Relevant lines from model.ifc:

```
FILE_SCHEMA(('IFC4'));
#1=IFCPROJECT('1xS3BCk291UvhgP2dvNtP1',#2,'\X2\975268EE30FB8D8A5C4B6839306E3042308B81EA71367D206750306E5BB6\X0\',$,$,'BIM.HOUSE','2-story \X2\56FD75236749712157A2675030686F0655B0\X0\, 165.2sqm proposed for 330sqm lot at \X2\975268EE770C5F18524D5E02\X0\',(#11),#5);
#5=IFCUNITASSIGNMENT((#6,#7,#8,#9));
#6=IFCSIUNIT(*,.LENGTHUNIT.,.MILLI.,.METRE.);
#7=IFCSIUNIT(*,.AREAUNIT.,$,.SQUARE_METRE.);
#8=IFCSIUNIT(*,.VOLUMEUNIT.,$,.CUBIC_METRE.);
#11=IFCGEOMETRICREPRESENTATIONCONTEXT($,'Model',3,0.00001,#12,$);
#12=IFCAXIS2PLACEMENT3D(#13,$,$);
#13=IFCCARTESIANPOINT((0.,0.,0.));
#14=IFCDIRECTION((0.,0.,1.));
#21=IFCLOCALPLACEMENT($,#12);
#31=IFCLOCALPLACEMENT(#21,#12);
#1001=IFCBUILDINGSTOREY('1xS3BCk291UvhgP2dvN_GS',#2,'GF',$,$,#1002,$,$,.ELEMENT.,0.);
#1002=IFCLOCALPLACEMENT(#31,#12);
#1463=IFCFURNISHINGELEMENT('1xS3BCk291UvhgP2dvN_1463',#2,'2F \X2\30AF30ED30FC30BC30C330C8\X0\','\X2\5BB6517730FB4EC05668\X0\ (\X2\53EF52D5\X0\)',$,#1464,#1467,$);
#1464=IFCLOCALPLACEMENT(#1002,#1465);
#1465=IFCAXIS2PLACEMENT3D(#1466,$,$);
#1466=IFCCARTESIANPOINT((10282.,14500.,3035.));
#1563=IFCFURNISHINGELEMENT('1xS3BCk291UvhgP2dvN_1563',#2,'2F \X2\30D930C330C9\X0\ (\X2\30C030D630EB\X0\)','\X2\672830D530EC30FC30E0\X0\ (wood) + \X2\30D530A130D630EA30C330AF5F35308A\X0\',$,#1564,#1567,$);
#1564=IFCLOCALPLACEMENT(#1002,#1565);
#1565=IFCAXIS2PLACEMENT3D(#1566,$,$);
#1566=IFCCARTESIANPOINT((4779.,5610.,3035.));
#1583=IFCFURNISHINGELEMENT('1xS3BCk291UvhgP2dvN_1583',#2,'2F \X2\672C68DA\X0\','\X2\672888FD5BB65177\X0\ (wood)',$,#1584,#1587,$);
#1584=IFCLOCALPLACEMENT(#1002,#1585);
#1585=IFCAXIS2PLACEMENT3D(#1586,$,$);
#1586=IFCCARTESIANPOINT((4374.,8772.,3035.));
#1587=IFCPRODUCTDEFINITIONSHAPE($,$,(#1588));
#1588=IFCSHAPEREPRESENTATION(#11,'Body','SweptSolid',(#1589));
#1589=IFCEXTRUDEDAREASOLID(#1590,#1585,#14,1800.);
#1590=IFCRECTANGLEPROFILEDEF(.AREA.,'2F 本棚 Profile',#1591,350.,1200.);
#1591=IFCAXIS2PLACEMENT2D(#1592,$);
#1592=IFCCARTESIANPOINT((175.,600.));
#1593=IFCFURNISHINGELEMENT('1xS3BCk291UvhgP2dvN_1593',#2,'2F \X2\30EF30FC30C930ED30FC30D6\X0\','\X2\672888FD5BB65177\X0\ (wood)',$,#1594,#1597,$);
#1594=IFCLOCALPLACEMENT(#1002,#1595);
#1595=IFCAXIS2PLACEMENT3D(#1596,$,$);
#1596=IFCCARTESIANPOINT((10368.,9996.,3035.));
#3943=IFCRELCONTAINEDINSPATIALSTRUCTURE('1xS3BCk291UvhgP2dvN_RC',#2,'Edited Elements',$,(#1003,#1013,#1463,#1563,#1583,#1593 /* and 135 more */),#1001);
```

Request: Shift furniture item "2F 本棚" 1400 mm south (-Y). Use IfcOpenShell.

```python
import ifcopenshell
import ifcopenshell.api.geometry
import ifcopenshell.util.placement
import ifcopenshell.util.unit

model = ifcopenshell.open("model.ifc")
unit_scale = ifcopenshell.util.unit.calculate_unit_scale(model)

item = model.by_guid("1xS3BCk291UvhgP2dvN_1583")
matrix = ifcopenshell.util.placement.get_local_placement(item.ObjectPlacement)
matrix[1, 3] -= 1.4 / unit_scale
ifcopenshell.api.geometry.edit_object_placement(model, product=item, matrix=matrix, is_si=False)

print(ifcopenshell.util.placement.get_local_placement(item.ObjectPlacement).round(3) + 0.0)

model.write("model_rev.ifc")
```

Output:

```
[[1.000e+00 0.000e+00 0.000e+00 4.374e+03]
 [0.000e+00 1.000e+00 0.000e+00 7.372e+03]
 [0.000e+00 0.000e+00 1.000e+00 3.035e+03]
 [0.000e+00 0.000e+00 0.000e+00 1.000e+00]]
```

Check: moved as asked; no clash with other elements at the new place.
